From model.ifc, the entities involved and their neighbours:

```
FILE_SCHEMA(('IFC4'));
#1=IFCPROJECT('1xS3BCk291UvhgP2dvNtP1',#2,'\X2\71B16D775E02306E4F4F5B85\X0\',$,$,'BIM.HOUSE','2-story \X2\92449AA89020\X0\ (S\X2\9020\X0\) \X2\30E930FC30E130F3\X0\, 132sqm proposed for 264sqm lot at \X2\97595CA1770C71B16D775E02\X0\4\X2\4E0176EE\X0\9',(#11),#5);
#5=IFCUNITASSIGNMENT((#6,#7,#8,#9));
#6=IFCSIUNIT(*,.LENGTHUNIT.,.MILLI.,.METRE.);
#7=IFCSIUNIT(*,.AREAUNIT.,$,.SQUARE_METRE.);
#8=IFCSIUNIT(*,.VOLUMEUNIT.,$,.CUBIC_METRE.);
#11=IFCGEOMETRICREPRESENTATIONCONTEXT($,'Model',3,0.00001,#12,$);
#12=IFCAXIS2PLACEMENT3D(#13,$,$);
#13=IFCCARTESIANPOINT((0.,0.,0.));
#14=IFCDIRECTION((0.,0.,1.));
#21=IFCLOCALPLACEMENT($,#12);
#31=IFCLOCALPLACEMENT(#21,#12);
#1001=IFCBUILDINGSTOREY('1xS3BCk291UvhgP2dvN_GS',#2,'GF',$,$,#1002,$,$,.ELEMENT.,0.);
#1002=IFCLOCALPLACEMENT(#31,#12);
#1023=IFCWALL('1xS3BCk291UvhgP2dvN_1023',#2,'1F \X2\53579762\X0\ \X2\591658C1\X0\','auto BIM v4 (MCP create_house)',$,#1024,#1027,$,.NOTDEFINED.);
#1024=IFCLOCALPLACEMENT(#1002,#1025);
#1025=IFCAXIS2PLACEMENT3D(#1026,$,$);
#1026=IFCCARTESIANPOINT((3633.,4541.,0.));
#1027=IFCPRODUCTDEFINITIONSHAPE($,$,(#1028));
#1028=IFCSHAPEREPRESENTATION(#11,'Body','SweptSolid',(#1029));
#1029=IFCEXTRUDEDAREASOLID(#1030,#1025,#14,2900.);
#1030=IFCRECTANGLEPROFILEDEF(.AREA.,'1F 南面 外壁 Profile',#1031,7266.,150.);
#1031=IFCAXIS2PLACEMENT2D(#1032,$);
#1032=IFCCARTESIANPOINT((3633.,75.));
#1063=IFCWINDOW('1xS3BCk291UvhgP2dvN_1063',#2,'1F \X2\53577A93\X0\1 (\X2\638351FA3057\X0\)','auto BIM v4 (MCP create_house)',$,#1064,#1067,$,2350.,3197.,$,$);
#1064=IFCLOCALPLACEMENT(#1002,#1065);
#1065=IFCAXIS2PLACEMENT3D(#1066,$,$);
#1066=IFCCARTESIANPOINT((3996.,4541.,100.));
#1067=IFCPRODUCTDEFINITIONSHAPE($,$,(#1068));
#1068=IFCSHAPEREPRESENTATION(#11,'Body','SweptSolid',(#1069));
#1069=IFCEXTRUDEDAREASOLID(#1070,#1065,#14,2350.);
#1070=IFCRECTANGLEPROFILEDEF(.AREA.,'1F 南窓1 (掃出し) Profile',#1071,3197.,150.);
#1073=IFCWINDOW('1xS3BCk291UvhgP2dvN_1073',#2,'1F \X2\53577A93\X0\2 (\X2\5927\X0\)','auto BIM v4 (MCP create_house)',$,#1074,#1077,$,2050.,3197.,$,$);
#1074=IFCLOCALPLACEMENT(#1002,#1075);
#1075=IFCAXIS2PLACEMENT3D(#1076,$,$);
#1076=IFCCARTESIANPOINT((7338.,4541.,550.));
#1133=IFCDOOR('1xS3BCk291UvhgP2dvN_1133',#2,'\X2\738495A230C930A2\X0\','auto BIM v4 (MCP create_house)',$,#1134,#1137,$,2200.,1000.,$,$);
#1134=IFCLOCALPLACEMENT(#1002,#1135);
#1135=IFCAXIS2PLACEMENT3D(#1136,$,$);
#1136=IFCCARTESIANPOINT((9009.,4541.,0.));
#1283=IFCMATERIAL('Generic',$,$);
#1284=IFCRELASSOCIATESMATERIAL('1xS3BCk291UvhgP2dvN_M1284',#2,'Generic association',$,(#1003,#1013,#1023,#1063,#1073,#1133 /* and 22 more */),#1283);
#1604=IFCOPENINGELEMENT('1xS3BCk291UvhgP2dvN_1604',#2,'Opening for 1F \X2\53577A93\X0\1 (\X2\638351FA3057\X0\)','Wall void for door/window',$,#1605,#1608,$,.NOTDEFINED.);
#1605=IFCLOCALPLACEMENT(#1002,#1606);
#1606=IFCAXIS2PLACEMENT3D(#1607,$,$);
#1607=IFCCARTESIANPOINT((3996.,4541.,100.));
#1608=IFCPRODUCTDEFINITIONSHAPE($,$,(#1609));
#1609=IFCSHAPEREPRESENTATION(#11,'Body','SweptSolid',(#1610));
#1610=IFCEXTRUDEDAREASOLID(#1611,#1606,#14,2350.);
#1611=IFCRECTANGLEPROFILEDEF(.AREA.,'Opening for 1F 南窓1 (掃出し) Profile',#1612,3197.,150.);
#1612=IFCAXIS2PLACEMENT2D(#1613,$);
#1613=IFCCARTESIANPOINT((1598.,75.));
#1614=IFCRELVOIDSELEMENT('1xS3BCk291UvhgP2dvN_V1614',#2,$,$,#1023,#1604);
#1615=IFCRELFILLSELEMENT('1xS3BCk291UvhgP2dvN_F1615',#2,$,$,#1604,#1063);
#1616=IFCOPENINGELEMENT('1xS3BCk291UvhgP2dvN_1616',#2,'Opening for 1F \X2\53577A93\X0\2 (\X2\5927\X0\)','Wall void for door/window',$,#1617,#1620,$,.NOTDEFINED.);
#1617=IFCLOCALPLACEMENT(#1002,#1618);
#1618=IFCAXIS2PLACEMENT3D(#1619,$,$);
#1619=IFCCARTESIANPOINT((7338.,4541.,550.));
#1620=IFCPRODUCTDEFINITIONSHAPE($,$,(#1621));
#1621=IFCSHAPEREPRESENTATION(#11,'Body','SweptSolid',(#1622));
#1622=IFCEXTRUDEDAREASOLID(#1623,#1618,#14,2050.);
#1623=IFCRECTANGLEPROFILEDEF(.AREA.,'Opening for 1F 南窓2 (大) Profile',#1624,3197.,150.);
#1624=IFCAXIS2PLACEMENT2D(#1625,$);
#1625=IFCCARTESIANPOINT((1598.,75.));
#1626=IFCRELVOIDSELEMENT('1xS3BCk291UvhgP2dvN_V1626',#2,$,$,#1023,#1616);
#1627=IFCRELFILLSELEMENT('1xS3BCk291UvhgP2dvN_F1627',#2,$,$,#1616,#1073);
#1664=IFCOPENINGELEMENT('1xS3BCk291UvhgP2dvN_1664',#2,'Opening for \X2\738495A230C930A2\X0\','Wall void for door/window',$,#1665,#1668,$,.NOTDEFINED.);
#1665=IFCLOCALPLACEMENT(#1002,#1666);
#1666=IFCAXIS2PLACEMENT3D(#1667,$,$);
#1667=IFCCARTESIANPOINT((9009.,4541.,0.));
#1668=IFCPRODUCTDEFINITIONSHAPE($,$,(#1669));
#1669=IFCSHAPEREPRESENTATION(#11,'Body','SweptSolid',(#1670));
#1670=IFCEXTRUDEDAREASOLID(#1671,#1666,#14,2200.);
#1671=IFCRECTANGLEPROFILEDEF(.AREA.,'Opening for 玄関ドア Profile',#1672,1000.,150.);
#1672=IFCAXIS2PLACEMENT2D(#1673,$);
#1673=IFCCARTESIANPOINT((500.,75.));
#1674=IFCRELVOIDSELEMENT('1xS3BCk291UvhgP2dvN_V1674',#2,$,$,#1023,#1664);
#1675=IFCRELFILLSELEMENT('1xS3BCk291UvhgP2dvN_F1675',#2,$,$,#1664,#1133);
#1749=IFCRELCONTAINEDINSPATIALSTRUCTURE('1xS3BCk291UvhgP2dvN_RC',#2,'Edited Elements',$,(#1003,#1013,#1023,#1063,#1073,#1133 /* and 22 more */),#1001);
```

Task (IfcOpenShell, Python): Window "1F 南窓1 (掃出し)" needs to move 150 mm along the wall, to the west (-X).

```python
import ifcopenshell
import ifcopenshell.api.geometry
import ifcopenshell.util.placement

model = ifcopenshell.open("model.ifc")

window = model.by_guid("1xS3BCk291UvhgP2dvN_1063")
opening = window.FillsVoids[0].RelatingOpeningElement
wall = opening.VoidsElements[0].RelatingBuildingElement

wall_matrix = ifcopenshell.util.placement.get_local_placement(wall.ObjectPlacement)
shift = wall_matrix[:3, 0] * -150.0
before = ifcopenshell.util.placement.get_local_placement(window.ObjectPlacement)[:3, 3].copy()

# The window is not placed relative to its opening, so move both.
for product in (opening, window):
    matrix = ifcopenshell.util.placement.get_local_placement(product.ObjectPlacement)
    matrix[:3, 3] += shift
    ifcopenshell.api.geometry.edit_object_placement(model, product=product, matrix=matrix, is_si=False)

after = ifcopenshell.util.placement.get_local_placement(window.ObjectPlacement)[:3, 3]
print("window moved by", (after - before).round(3) + 0.0)

model.write("model_updated.ifc")
```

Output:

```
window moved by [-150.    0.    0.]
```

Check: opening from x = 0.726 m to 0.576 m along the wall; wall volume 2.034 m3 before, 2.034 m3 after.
